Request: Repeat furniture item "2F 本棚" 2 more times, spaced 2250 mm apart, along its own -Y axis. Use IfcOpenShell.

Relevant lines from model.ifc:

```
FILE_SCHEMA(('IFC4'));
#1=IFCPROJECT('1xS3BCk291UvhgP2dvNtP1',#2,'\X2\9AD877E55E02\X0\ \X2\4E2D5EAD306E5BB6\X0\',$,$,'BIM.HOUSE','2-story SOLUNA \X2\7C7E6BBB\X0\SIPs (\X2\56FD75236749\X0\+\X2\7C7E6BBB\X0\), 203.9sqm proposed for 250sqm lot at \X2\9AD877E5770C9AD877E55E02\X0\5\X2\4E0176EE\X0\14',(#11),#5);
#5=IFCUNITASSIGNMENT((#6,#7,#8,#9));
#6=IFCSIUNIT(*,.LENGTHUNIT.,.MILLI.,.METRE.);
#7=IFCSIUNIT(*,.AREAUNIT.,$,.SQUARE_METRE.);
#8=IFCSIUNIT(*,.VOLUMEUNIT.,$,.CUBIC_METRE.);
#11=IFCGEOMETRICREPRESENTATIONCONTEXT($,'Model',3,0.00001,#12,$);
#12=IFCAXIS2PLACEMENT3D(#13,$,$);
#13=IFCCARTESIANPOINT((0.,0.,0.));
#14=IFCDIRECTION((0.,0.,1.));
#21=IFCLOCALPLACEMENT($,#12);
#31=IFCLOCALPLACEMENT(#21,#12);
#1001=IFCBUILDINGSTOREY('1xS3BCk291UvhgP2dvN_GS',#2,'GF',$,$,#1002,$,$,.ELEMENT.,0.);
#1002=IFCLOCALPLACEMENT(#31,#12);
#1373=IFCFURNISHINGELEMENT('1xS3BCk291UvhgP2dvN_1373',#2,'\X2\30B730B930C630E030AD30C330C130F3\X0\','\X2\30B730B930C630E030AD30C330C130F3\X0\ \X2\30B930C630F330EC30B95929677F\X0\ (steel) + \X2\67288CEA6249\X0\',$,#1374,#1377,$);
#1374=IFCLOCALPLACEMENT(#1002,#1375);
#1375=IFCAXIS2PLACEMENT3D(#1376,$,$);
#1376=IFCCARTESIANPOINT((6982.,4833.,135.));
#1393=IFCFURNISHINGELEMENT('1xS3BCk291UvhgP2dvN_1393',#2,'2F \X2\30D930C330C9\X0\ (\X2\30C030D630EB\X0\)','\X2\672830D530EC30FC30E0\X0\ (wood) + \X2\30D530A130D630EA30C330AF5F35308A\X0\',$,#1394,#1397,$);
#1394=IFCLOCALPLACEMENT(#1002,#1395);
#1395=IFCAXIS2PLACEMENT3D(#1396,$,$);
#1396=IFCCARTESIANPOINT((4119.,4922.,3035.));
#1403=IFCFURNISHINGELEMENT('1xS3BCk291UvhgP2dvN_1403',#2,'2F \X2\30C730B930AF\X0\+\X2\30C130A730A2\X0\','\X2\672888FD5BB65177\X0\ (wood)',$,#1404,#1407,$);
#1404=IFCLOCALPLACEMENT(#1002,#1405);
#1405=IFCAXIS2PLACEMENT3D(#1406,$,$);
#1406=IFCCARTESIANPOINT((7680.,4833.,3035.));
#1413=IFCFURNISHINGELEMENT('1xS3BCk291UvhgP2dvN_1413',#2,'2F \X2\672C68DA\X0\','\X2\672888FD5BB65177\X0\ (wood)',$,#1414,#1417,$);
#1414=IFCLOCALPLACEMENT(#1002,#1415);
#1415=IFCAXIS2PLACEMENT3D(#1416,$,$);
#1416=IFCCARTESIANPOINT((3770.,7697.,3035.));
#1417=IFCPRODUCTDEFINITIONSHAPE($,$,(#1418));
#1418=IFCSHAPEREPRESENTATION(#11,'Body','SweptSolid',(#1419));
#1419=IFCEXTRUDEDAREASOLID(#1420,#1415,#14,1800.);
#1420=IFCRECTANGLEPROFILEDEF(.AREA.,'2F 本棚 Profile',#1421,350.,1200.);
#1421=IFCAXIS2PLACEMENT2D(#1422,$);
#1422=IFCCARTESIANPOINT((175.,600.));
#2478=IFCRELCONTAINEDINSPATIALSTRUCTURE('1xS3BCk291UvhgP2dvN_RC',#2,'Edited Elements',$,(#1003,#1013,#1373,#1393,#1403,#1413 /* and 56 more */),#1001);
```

```python
import ifcopenshell
import ifcopenshell.api.geometry
import ifcopenshell.api.root
import ifcopenshell.util.element
import ifcopenshell.util.placement

model = ifcopenshell.open("model.ifc")


def reuse_history(source, copy):
    """copy_class also copies each property set's owner history, people and application; keep the originals."""
    for rel in copy.IsDefinedBy:
        if rel.is_a("IfcRelDefinesByProperties") and (history := rel.RelatingPropertyDefinition.OwnerHistory):
            rel.RelatingPropertyDefinition.OwnerHistory = source.OwnerHistory
            ifcopenshell.util.element.remove_deep2(model, history)


source = model.by_id(1413)
base = ifcopenshell.util.placement.get_local_placement(source.ObjectPlacement)
step = -base[:3, 1] * 2250.0

for i in range(1, 3):
    copy = ifcopenshell.api.root.copy_class(model, product=source)
    copy.Representation = ifcopenshell.util.element.copy_deep(
        model, source.Representation, exclude=["IfcGeometricRepresentationContext", "IfcRepresentationMap"]
    )
    reuse_history(source, copy)
    matrix = base.copy()
    matrix[:3, 3] += i * step
    print("added at", matrix[:3, 3].round(3) + 0.0)
    ifcopenshell.api.geometry.edit_object_placement(model, product=copy, matrix=matrix, is_si=False)

model.write("model-out.ifc")
```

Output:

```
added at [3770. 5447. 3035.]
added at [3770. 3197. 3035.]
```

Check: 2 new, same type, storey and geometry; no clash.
